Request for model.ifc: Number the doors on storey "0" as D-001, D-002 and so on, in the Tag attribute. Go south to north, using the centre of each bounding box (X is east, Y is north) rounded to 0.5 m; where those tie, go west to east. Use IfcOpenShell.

First a look at what the model holds.

```python
import ifcopenshell
import ifcopenshell.util.element
import ifcopenshell.util.placement

model = ifcopenshell.open("model.ifc")
print(model.schema)
storey = next(s for s in model.by_type("IfcBuildingStorey") if s.Name == "0")
doors = [e for e in ifcopenshell.util.element.get_decomposition(storey) if e.is_a("IfcDoor")]
for e in sorted(doors, key=lambda e: e.id()):
    origin = ifcopenshell.util.placement.get_local_placement(e.ObjectPlacement)[:3, 3]
    print(e.id(), e.Tag, e.Name, origin.round(2) + 0.0, sep=" | ")
```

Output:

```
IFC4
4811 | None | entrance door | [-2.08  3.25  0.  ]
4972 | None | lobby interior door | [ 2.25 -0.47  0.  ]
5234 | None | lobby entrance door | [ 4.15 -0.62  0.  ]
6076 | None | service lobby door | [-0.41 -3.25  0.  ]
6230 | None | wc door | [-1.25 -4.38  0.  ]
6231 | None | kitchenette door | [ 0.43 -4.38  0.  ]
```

```python
import ifcopenshell
import ifcopenshell.geom
import ifcopenshell.util.element
import ifcopenshell.util.shape

model = ifcopenshell.open("model.ifc")
settings = ifcopenshell.geom.settings()
settings.set("use-world-coords", True)


def centre(element):
    shape = ifcopenshell.geom.create_shape(settings, element)
    return ifcopenshell.util.shape.get_bbox_centroid(shape.geometry)


storey = next(s for s in model.by_type("IfcBuildingStorey") if s.Name == "0")
doors = [e for e in ifcopenshell.util.element.get_decomposition(storey) if e.is_a("IfcDoor")]

# Insertion points can sit at a corner or the storey origin, so sort by the geometry (in metres).
centres = {e: centre(e) for e in doors}
doors.sort(key=lambda e: (round(centres[e][1] / 0.5), centres[e][0]))

for i, e in enumerate(doors, start=1):
    number = f"D-0{i:02d}"
    e.Tag = number
    print(e.id(), number)

model.write("model_updated.ifc")
```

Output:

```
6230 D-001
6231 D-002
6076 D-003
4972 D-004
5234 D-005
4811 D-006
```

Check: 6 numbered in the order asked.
